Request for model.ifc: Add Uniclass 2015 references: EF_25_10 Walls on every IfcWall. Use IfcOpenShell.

First a look at what the model holds.

```python
import ifcopenshell

model = ifcopenshell.open("model.ifc")
print(model.schema)
print("classifications:", [c.Name for c in model.by_type("IfcClassification")])
for ifc_class in ("IfcDoor", "IfcRoof", "IfcStair", "IfcWall", "IfcWindow"):
    print(ifc_class, len(model.by_type(ifc_class)))
```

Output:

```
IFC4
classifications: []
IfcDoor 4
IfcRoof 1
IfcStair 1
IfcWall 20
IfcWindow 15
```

```python
import ifcopenshell
import ifcopenshell.api.classification

model = ifcopenshell.open("model.ifc")

system = ifcopenshell.api.classification.add_classification(model, classification="Uniclass 2015")

codes = {
    "IfcWall": ("EF_25_10", "Walls"),
}
for ifc_class, (code, name) in codes.items():
    products = model.by_type(ifc_class)
    ifcopenshell.api.classification.add_reference(
        model, products=products, classification=system, identification=code, name=name
    )
    print(code, len(products))

model.write("model_updated.ifc")
```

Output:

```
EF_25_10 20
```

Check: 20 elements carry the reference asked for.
